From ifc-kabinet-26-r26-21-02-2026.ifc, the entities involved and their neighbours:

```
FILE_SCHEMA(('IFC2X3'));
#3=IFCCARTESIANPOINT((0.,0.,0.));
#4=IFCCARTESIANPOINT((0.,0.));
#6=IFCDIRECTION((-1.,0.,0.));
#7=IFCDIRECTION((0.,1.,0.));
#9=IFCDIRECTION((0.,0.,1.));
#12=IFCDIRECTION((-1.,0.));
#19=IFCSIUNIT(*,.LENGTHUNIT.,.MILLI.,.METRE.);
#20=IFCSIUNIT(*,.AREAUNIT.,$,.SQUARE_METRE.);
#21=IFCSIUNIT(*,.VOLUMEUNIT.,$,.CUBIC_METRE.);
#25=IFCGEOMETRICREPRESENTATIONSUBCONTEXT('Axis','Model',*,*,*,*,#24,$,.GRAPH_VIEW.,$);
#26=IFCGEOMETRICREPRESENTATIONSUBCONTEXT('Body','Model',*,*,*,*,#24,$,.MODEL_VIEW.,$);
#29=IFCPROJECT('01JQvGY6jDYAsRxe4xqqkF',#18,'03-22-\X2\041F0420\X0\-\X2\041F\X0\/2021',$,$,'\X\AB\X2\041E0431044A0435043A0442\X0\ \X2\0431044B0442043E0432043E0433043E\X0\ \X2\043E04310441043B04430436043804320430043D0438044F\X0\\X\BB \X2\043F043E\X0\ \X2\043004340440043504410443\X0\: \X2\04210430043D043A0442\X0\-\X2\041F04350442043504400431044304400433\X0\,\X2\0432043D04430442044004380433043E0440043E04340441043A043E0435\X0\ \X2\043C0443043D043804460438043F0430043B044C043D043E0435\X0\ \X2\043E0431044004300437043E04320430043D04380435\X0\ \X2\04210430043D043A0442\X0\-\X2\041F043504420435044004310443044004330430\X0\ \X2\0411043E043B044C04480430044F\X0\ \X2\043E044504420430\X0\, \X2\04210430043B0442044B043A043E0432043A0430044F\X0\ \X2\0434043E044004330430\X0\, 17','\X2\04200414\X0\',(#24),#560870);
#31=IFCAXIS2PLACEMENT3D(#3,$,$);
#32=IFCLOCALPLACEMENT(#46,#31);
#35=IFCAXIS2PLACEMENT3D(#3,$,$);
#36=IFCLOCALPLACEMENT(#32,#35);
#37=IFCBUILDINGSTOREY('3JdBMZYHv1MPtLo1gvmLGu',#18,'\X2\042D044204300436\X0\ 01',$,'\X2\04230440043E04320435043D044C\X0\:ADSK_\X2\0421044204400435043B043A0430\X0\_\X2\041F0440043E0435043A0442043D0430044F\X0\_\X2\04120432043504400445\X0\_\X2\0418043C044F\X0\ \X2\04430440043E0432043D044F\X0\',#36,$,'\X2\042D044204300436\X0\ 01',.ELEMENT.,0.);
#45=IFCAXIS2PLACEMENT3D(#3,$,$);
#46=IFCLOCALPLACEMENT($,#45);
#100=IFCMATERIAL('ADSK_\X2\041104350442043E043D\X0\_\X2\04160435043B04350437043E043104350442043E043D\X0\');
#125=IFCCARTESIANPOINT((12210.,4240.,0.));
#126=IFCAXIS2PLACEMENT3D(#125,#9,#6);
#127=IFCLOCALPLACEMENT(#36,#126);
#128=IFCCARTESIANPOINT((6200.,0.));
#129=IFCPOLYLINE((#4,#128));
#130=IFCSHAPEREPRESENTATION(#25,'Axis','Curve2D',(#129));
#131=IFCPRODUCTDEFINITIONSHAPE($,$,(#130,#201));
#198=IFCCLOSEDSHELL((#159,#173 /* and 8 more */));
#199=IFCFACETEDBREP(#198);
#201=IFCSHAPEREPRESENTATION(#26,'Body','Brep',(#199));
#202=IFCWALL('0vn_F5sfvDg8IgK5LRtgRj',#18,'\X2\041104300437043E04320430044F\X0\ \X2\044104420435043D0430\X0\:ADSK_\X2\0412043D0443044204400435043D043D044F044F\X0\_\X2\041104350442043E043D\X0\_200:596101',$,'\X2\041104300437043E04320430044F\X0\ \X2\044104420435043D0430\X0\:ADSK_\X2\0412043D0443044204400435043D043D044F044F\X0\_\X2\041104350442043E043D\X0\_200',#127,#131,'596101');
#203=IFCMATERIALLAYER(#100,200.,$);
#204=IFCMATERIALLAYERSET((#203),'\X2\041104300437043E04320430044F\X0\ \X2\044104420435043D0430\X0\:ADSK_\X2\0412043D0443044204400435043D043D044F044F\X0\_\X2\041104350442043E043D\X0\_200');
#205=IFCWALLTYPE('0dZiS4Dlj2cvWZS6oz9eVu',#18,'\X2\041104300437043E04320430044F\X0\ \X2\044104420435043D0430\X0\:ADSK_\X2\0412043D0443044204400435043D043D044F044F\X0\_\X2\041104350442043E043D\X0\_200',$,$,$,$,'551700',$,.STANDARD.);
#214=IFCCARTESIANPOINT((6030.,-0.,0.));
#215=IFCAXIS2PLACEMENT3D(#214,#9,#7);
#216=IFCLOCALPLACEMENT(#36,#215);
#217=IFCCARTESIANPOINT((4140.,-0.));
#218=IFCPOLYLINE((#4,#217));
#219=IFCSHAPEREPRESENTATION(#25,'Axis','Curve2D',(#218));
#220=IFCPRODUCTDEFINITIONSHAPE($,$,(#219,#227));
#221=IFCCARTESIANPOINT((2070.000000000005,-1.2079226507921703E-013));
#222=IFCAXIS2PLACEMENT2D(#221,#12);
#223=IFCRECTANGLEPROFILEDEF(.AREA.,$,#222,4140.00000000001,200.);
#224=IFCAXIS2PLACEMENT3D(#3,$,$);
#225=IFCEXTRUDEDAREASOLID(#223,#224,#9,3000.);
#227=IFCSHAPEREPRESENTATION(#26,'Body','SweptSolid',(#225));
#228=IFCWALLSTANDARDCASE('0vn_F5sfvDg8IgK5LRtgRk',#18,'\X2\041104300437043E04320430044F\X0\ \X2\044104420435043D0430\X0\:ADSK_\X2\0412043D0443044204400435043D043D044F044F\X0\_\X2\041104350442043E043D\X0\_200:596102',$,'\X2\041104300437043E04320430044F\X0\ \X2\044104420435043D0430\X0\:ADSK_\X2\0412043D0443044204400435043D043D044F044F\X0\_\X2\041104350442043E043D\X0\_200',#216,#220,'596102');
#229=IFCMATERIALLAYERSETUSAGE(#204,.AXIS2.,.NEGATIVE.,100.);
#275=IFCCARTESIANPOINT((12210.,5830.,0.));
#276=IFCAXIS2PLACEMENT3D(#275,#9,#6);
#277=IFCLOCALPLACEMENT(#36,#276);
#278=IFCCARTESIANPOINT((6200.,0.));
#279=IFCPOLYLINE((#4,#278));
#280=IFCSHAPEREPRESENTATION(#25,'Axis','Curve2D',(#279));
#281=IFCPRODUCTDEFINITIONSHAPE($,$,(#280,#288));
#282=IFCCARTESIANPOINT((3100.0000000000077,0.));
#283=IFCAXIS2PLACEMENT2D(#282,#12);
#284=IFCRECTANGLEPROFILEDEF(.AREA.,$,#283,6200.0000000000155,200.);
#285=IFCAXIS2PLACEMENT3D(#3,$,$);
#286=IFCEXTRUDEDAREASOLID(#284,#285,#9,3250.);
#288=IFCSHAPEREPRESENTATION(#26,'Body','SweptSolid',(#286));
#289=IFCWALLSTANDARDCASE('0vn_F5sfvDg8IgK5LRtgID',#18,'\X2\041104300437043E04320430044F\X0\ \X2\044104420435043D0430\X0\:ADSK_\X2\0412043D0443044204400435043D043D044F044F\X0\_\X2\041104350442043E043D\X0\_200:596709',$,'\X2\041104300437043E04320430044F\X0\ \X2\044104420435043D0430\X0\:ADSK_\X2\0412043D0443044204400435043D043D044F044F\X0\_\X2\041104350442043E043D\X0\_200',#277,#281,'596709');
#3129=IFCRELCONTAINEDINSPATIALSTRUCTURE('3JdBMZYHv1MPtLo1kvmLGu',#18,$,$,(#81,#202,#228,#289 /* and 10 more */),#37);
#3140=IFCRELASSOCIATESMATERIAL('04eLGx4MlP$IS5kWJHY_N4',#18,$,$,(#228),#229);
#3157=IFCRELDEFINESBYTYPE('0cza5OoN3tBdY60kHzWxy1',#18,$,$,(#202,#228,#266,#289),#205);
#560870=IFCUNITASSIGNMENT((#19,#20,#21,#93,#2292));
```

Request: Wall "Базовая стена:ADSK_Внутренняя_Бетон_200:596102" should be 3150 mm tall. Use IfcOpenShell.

```python
import ifcopenshell
import ifcopenshell.geom
import ifcopenshell.util.representation
import ifcopenshell.util.shape

model = ifcopenshell.open("ifc-kabinet-26-r26-21-02-2026.ifc")
settings = ifcopenshell.geom.settings()


def volume(element):
    """Net volume in cubic metres, openings subtracted."""
    shape = ifcopenshell.geom.create_shape(settings, element)
    return ifcopenshell.util.shape.get_volume(shape.geometry)


wall = model.by_guid("0vn_F5sfvDg8IgK5LRtgRk")
before = volume(wall)

body = ifcopenshell.util.representation.get_representation(wall, "Model", "Body")
solid = body.Items[0]
old_height = solid.Depth
solid.Depth = 3150.0
after = volume(wall)

print(f"height {old_height:g} -> {solid.Depth:g}, volume {before:.3f} -> {after:.3f} m3")

model.write("ifc-kabinet-26-r26-21-02-2026_updated.ifc")
```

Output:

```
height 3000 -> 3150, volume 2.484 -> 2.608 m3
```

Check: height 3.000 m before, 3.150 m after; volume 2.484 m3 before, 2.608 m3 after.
